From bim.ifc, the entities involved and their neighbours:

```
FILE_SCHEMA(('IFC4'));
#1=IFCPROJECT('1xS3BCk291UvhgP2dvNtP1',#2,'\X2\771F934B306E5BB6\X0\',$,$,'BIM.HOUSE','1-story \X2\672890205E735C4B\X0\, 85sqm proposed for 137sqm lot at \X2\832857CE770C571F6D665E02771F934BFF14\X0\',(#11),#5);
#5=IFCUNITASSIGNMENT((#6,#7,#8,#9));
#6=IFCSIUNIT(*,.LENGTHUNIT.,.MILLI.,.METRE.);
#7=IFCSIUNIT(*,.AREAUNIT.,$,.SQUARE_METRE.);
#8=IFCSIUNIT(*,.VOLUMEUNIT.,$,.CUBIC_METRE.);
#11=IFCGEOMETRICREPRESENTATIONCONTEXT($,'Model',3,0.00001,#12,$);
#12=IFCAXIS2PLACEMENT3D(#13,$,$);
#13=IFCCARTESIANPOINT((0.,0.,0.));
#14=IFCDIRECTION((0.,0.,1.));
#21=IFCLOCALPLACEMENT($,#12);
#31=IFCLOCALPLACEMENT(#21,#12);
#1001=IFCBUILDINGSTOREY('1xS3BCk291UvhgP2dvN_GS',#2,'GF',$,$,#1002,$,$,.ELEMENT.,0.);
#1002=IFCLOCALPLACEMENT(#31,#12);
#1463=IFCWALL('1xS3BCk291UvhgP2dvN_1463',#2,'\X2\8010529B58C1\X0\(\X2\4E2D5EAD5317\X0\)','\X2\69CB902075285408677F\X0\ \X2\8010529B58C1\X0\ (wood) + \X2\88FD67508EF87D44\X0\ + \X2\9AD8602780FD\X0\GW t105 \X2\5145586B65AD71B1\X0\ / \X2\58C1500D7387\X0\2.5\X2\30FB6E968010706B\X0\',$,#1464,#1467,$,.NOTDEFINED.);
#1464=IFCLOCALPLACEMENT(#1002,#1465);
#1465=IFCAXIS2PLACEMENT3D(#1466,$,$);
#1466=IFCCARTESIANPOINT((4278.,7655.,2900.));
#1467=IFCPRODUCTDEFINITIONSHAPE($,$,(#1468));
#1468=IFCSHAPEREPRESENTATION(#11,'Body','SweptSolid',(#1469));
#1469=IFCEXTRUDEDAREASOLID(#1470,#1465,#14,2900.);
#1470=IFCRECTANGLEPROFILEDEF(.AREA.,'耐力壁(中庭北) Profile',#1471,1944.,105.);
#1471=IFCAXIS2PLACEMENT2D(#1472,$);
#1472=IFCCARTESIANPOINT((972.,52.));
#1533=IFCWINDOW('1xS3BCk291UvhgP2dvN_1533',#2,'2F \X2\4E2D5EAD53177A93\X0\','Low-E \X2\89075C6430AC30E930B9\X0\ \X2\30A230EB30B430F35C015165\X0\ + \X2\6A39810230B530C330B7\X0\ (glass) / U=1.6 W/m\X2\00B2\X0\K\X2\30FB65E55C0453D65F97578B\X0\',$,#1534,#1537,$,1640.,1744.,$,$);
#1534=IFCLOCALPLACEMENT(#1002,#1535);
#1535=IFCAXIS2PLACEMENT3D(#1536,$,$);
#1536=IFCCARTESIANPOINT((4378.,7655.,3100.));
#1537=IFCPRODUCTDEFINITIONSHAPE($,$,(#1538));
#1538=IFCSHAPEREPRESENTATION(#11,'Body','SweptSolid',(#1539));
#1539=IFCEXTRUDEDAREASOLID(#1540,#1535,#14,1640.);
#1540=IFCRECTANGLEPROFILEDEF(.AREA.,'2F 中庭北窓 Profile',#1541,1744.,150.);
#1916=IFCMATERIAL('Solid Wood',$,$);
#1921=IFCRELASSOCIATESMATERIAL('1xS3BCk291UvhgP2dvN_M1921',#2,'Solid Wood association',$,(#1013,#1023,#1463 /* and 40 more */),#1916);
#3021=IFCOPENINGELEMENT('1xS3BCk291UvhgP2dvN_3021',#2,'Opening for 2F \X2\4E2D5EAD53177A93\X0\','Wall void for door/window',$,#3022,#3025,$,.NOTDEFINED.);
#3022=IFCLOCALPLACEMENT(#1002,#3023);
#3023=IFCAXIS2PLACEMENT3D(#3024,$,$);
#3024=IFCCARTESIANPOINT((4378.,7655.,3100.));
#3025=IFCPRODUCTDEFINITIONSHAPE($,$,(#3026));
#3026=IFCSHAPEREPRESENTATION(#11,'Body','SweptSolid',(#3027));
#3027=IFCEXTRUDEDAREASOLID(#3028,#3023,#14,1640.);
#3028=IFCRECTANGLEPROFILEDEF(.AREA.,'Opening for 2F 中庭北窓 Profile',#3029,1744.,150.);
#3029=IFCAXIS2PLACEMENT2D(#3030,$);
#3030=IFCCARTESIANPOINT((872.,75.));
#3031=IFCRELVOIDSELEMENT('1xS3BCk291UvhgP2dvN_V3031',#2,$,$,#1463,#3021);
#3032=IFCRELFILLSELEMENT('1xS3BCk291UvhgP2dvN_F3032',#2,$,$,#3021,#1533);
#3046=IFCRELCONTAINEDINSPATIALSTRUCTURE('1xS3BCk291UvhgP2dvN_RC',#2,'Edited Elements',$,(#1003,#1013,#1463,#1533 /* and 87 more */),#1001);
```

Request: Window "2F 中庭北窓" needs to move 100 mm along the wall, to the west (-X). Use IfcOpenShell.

```python
import ifcopenshell
import ifcopenshell.api.geometry
import ifcopenshell.util.placement
import ifcopenshell.util.unit

model = ifcopenshell.open("bim.ifc")
unit_scale = ifcopenshell.util.unit.calculate_unit_scale(model)

window = model.by_guid("1xS3BCk291UvhgP2dvN_1533")
opening = window.FillsVoids[0].RelatingOpeningElement
wall = opening.VoidsElements[0].RelatingBuildingElement

wall_matrix = ifcopenshell.util.placement.get_local_placement(wall.ObjectPlacement)
shift = wall_matrix[:3, 0] * -0.1 / unit_scale
before = ifcopenshell.util.placement.get_local_placement(window.ObjectPlacement)[:3, 3].copy()

# The window is not placed relative to its opening, so move both.
for product in (opening, window):
    matrix = ifcopenshell.util.placement.get_local_placement(product.ObjectPlacement)
    matrix[:3, 3] += shift
    ifcopenshell.api.geometry.edit_object_placement(model, product=product, matrix=matrix, is_si=False)

after = ifcopenshell.util.placement.get_local_placement(window.ObjectPlacement)[:3, 3]
print("window moved by", (after - before).round(3) + 0.0)

model.write("bim_v2.ifc")
```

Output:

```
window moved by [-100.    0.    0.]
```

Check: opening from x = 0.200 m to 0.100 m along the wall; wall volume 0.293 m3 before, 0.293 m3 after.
